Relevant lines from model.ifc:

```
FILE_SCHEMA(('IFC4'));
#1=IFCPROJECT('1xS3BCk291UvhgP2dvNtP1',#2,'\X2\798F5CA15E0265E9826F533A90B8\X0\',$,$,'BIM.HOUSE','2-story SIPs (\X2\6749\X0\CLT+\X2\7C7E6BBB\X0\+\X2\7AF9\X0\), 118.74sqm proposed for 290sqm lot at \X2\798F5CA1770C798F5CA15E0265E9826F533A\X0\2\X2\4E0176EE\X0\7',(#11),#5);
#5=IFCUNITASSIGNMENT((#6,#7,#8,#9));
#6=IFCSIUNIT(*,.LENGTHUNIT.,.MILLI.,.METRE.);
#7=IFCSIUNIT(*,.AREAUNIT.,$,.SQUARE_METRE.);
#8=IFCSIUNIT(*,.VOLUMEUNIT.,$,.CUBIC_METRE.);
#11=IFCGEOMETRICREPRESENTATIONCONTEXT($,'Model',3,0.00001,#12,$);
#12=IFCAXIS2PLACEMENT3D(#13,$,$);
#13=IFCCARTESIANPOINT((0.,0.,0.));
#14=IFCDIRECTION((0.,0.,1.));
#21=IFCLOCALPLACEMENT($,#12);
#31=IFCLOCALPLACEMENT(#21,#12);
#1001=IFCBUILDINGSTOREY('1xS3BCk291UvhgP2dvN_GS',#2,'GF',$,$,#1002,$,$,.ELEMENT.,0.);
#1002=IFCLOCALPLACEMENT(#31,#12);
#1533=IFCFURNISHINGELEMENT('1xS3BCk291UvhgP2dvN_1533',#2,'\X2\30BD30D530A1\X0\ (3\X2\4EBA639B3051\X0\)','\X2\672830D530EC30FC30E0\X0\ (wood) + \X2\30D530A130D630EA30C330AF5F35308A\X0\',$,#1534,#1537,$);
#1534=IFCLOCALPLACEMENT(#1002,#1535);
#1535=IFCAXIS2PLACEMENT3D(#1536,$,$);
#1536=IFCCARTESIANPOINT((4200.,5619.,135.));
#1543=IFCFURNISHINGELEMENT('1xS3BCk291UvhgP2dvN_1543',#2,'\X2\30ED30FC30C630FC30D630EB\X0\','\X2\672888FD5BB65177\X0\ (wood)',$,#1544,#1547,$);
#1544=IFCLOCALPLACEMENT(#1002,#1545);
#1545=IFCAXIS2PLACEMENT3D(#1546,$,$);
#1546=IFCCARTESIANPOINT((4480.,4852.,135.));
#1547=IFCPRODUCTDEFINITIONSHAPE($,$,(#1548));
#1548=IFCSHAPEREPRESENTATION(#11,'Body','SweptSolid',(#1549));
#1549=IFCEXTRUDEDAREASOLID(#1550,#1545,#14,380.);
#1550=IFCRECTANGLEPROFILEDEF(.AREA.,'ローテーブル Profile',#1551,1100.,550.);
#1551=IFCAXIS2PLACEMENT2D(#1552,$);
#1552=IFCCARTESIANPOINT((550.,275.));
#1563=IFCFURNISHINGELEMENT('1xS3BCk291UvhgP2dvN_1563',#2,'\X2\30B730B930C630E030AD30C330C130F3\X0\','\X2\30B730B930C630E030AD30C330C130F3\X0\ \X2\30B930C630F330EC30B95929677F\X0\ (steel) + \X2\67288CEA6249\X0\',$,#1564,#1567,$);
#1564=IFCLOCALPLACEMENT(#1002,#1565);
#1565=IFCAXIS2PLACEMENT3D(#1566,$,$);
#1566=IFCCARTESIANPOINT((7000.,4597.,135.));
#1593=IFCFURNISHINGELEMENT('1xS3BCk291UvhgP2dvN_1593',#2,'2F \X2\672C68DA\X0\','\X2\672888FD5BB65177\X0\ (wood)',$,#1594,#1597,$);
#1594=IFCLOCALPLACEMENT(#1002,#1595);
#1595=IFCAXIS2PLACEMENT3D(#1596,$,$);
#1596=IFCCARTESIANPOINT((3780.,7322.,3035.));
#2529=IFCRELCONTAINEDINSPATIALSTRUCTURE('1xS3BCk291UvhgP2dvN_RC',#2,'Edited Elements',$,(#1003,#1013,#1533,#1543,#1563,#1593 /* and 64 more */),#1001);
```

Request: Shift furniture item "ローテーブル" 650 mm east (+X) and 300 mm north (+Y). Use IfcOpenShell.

```python
import ifcopenshell
import ifcopenshell.api.geometry
import ifcopenshell.util.placement
import ifcopenshell.util.unit

model = ifcopenshell.open("model.ifc")
unit_scale = ifcopenshell.util.unit.calculate_unit_scale(model)

item = model.by_id(1543)
matrix = ifcopenshell.util.placement.get_local_placement(item.ObjectPlacement)
matrix[0, 3] += 0.65 / unit_scale
matrix[1, 3] += 0.3 / unit_scale
ifcopenshell.api.geometry.edit_object_placement(model, product=item, matrix=matrix, is_si=False)

print(ifcopenshell.util.placement.get_local_placement(item.ObjectPlacement).round(3) + 0.0)

model.write("model_updated.ifc")
```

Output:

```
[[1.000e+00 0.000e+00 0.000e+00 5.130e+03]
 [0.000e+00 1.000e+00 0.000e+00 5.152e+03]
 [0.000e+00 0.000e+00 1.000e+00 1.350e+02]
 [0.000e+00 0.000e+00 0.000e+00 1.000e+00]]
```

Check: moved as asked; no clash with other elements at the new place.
